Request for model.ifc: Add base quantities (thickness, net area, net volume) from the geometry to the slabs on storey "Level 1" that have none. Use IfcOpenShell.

First a look at what the model holds.

```python
import ifcopenshell
import ifcopenshell.util.element
import ifcopenshell.util.unit

model = ifcopenshell.open("model.ifc")
print(model.schema)
for unit_type in ("LENGTHUNIT", "AREAUNIT", "VOLUMEUNIT"):
    print(unit_type, ifcopenshell.util.unit.calculate_unit_scale(model, unit_type))
storey = next(s for s in model.by_type("IfcBuildingStorey") if s.Name == "Level 1")
slabs = [e for e in ifcopenshell.util.element.get_decomposition(storey) if e.is_a("IfcSlab")]
for e in sorted(slabs, key=lambda e: e.id()):
    print(e.id(), e.is_a(), e.Name, list(ifcopenshell.util.element.get_psets(e, qtos_only=True)), sep=" | ")
```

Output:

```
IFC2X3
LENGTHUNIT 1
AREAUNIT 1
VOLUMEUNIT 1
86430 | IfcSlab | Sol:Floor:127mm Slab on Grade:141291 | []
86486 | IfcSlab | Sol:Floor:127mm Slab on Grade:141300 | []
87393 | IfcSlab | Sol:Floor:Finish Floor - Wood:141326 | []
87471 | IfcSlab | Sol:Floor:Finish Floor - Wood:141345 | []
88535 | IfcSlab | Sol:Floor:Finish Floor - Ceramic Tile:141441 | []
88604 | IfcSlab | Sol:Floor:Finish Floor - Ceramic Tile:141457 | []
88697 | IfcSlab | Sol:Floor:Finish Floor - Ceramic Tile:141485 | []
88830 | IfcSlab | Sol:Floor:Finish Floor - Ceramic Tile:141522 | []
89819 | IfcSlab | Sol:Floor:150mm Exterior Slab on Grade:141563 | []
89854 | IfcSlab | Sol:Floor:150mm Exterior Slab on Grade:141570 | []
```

```python
import ifcopenshell
import ifcopenshell.api.pset
import ifcopenshell.geom
import ifcopenshell.util.element
import ifcopenshell.util.shape
import ifcopenshell.util.unit

model = ifcopenshell.open("model.ifc")
unit_scale = ifcopenshell.util.unit.calculate_unit_scale(model)
area_scale = ifcopenshell.util.unit.calculate_unit_scale(model, "AREAUNIT")
volume_scale = ifcopenshell.util.unit.calculate_unit_scale(model, "VOLUMEUNIT")
settings = ifcopenshell.geom.settings()

storey = next(s for s in model.by_type("IfcBuildingStorey") if s.Name == "Level 1")
slabs = [e for e in ifcopenshell.util.element.get_decomposition(storey) if e.is_a("IfcSlab")]

for e in sorted(slabs, key=lambda e: e.id()):
    if ifcopenshell.util.element.get_psets(e, qtos_only=True, should_inherit=False):
        continue
    # Geometry comes back in metres, in the element's own axes.
    shape = ifcopenshell.geom.create_shape(settings, e)
    values = {
        "Width": ifcopenshell.util.shape.get_z(shape.geometry) / unit_scale,
        "NetArea": ifcopenshell.util.shape.get_footprint_area(shape.geometry) / area_scale,
        "NetVolume": ifcopenshell.util.shape.get_volume(shape.geometry) / volume_scale,
    }
    qto = ifcopenshell.api.pset.add_qto(model, product=e, name="BaseQuantities")
    ifcopenshell.api.pset.edit_qto(model, qto=qto, properties=values)
    print(e.id(), {k: round(v, 3) for k, v in values.items()})

model.write("model_updated.ifc")
```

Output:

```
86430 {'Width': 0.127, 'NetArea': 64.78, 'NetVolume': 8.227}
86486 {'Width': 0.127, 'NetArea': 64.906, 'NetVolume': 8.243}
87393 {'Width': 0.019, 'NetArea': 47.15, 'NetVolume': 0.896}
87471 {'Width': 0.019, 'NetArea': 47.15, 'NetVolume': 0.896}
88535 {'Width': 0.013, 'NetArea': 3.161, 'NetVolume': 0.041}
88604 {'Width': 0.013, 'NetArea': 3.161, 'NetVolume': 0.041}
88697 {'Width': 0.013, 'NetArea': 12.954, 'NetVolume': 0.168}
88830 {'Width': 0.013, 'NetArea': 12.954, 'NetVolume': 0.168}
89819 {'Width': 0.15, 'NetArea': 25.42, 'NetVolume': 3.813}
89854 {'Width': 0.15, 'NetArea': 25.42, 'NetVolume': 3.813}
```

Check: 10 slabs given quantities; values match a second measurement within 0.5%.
